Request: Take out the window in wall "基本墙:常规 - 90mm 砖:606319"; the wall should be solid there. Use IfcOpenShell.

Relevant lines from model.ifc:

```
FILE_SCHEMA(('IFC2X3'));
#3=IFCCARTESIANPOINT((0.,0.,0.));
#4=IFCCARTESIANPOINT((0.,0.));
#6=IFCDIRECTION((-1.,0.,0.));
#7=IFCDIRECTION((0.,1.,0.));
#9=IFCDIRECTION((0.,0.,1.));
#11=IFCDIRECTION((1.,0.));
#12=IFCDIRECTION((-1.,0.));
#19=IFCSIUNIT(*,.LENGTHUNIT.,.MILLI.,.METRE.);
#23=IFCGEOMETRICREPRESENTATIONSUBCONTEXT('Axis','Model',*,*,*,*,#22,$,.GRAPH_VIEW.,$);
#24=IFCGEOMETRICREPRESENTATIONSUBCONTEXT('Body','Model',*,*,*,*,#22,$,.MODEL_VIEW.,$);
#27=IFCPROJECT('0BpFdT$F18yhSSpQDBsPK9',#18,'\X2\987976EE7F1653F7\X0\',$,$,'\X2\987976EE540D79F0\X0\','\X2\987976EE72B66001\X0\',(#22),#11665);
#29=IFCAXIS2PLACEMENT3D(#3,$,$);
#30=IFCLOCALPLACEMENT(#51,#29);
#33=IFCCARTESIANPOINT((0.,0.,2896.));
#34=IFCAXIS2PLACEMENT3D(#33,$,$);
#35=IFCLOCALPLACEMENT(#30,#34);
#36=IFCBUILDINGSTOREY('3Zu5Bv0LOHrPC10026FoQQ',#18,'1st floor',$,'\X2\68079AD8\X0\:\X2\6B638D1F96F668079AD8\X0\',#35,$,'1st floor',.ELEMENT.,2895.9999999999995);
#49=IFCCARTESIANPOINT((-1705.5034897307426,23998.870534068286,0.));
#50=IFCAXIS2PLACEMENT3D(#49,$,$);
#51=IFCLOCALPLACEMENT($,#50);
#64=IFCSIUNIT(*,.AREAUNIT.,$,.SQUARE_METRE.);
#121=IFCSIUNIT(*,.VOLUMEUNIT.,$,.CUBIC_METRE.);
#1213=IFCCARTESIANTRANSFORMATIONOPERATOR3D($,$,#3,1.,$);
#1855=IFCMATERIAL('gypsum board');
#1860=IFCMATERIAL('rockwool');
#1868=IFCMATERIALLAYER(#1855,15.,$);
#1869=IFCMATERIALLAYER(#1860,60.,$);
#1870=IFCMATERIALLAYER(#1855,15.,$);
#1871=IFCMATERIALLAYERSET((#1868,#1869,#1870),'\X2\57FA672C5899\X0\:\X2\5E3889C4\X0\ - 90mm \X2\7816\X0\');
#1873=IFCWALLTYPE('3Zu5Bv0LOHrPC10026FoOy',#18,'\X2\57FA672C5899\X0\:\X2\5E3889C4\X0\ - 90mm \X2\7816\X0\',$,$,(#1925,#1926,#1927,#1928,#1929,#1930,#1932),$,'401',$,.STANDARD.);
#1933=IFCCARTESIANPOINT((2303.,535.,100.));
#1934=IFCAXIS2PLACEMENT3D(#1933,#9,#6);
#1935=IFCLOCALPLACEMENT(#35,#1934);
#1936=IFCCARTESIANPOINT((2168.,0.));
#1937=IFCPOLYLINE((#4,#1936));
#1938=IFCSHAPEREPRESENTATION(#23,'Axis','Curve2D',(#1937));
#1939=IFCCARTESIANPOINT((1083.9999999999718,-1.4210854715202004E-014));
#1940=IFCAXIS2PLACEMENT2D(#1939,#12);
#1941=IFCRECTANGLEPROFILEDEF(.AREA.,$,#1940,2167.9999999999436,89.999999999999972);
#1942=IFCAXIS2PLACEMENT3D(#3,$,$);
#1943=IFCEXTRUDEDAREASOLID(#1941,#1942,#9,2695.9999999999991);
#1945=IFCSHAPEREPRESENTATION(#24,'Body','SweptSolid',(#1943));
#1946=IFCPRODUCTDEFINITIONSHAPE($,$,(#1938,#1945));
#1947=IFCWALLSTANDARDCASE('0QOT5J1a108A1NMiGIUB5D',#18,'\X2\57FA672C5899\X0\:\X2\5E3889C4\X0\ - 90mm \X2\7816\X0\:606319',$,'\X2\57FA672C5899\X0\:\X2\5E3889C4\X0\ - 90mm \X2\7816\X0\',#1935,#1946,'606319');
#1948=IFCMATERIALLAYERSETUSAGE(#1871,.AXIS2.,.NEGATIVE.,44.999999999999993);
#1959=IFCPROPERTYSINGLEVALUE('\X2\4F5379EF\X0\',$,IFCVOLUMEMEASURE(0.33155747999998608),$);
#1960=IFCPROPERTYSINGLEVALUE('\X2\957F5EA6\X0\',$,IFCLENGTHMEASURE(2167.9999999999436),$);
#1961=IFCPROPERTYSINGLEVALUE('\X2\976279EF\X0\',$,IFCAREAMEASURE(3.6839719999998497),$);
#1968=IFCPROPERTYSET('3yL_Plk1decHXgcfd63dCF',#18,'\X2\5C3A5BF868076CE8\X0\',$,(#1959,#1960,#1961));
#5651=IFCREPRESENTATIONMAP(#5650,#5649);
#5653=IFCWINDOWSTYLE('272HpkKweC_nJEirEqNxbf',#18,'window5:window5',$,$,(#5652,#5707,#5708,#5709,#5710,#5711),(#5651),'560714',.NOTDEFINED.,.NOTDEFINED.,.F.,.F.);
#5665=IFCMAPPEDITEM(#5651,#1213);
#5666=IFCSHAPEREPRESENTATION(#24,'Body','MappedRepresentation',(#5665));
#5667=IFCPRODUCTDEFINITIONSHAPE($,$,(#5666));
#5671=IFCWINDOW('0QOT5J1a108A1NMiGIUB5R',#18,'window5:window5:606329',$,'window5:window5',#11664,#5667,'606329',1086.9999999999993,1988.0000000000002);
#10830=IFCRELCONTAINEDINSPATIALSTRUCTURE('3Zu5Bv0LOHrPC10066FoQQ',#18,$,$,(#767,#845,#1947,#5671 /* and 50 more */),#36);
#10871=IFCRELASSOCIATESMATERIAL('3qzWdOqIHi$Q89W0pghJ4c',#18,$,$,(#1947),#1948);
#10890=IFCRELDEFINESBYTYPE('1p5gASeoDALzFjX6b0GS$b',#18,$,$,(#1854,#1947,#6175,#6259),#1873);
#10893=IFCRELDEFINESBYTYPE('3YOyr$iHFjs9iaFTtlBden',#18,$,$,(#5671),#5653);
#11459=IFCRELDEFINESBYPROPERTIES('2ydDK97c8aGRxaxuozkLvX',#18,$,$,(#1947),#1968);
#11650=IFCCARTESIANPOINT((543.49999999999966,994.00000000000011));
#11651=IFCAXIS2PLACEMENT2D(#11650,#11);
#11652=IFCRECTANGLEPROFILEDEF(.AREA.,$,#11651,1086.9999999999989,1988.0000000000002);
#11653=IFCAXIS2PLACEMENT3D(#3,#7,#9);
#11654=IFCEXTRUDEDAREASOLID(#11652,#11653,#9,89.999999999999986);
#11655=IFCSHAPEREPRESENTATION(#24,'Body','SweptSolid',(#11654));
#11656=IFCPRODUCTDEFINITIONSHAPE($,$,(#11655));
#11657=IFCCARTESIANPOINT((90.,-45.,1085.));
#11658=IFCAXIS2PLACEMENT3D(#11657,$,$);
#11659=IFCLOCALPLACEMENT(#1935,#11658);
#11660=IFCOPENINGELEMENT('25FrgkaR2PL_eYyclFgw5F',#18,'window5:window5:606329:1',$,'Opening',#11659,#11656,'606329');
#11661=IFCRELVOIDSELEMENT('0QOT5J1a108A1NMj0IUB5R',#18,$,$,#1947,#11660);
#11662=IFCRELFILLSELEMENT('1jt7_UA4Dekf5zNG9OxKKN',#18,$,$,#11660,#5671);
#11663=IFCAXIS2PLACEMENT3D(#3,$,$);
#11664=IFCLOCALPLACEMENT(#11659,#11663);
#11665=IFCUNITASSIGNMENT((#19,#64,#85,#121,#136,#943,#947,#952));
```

```python
import ifcopenshell
import ifcopenshell.api.feature
import ifcopenshell.api.pset
import ifcopenshell.api.root
import ifcopenshell.geom
import ifcopenshell.util.element
import ifcopenshell.util.shape
import ifcopenshell.util.unit

model = ifcopenshell.open("model.ifc")
area_scale = ifcopenshell.util.unit.calculate_unit_scale(model, "AREAUNIT")
volume_scale = ifcopenshell.util.unit.calculate_unit_scale(model, "VOLUMEUNIT")
settings = ifcopenshell.geom.settings()


def volume(element):
    """Net volume in cubic metres, openings subtracted."""
    shape = ifcopenshell.geom.create_shape(settings, element)
    return ifcopenshell.util.shape.get_volume(shape.geometry)


window = model.by_guid("0QOT5J1a108A1NMiGIUB5R")
opening = window.FillsVoids[0].RelatingOpeningElement
wall = opening.VoidsElements[0].RelatingBuildingElement
before = volume(wall)

ifcopenshell.api.root.remove_product(model, product=window)
ifcopenshell.api.feature.remove_feature(model, feature=opening)

after = volume(wall)
thickness = 0.09  # wall thickness in metres

# Update the wall's stored quantities.
pset = model.by_id(ifcopenshell.util.element.get_pset(wall, "尺寸标注", should_inherit=False)["id"])
ifcopenshell.api.pset.edit_pset(model, pset=pset, properties={
    "体积": model.create_entity("IfcVolumeMeasure", after / volume_scale),
    "面积": model.create_entity("IfcAreaMeasure", after / thickness / area_scale),
})

print(f"wall volume {before:.3f} -> {after:.3f} m3")

model.write("model-out.ifc")
```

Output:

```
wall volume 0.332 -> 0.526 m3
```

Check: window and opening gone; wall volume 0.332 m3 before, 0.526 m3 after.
